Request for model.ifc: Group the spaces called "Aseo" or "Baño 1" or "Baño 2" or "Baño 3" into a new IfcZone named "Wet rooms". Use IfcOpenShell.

First a look at what the model holds.

```python
import ifcopenshell

model = ifcopenshell.open("model.ifc")
print(model.schema)
seen = {}
for space in model.by_type("IfcSpace"):
    seen[space.LongName] = seen.get(space.LongName, 0) + 1
for name, count in sorted(seen.items(), key=str):
    print(count, "x", name)
print("zones:", [z.Name for z in model.by_type("IfcZone")][:20])
```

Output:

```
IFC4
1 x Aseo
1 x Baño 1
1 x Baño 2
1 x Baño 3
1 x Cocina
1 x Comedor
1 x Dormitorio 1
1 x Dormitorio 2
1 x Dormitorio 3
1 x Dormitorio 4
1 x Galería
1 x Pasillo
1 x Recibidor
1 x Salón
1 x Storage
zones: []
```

```python
import ifcopenshell
import ifcopenshell.api.group
import ifcopenshell.api.root

model = ifcopenshell.open("model.ifc")

names = {"Aseo", "Baño 1", "Baño 2", "Baño 3"}
spaces = [s for s in model.by_type("IfcSpace") if s.LongName in names]

zone = ifcopenshell.api.root.create_entity(model, ifc_class="IfcZone", name="Wet rooms")
ifcopenshell.api.group.assign_group(model, products=spaces, group=zone)
print(len(spaces), "spaces in", zone.Name)

model.write("model_edited.ifc")
```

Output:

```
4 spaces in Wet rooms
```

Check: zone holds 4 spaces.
